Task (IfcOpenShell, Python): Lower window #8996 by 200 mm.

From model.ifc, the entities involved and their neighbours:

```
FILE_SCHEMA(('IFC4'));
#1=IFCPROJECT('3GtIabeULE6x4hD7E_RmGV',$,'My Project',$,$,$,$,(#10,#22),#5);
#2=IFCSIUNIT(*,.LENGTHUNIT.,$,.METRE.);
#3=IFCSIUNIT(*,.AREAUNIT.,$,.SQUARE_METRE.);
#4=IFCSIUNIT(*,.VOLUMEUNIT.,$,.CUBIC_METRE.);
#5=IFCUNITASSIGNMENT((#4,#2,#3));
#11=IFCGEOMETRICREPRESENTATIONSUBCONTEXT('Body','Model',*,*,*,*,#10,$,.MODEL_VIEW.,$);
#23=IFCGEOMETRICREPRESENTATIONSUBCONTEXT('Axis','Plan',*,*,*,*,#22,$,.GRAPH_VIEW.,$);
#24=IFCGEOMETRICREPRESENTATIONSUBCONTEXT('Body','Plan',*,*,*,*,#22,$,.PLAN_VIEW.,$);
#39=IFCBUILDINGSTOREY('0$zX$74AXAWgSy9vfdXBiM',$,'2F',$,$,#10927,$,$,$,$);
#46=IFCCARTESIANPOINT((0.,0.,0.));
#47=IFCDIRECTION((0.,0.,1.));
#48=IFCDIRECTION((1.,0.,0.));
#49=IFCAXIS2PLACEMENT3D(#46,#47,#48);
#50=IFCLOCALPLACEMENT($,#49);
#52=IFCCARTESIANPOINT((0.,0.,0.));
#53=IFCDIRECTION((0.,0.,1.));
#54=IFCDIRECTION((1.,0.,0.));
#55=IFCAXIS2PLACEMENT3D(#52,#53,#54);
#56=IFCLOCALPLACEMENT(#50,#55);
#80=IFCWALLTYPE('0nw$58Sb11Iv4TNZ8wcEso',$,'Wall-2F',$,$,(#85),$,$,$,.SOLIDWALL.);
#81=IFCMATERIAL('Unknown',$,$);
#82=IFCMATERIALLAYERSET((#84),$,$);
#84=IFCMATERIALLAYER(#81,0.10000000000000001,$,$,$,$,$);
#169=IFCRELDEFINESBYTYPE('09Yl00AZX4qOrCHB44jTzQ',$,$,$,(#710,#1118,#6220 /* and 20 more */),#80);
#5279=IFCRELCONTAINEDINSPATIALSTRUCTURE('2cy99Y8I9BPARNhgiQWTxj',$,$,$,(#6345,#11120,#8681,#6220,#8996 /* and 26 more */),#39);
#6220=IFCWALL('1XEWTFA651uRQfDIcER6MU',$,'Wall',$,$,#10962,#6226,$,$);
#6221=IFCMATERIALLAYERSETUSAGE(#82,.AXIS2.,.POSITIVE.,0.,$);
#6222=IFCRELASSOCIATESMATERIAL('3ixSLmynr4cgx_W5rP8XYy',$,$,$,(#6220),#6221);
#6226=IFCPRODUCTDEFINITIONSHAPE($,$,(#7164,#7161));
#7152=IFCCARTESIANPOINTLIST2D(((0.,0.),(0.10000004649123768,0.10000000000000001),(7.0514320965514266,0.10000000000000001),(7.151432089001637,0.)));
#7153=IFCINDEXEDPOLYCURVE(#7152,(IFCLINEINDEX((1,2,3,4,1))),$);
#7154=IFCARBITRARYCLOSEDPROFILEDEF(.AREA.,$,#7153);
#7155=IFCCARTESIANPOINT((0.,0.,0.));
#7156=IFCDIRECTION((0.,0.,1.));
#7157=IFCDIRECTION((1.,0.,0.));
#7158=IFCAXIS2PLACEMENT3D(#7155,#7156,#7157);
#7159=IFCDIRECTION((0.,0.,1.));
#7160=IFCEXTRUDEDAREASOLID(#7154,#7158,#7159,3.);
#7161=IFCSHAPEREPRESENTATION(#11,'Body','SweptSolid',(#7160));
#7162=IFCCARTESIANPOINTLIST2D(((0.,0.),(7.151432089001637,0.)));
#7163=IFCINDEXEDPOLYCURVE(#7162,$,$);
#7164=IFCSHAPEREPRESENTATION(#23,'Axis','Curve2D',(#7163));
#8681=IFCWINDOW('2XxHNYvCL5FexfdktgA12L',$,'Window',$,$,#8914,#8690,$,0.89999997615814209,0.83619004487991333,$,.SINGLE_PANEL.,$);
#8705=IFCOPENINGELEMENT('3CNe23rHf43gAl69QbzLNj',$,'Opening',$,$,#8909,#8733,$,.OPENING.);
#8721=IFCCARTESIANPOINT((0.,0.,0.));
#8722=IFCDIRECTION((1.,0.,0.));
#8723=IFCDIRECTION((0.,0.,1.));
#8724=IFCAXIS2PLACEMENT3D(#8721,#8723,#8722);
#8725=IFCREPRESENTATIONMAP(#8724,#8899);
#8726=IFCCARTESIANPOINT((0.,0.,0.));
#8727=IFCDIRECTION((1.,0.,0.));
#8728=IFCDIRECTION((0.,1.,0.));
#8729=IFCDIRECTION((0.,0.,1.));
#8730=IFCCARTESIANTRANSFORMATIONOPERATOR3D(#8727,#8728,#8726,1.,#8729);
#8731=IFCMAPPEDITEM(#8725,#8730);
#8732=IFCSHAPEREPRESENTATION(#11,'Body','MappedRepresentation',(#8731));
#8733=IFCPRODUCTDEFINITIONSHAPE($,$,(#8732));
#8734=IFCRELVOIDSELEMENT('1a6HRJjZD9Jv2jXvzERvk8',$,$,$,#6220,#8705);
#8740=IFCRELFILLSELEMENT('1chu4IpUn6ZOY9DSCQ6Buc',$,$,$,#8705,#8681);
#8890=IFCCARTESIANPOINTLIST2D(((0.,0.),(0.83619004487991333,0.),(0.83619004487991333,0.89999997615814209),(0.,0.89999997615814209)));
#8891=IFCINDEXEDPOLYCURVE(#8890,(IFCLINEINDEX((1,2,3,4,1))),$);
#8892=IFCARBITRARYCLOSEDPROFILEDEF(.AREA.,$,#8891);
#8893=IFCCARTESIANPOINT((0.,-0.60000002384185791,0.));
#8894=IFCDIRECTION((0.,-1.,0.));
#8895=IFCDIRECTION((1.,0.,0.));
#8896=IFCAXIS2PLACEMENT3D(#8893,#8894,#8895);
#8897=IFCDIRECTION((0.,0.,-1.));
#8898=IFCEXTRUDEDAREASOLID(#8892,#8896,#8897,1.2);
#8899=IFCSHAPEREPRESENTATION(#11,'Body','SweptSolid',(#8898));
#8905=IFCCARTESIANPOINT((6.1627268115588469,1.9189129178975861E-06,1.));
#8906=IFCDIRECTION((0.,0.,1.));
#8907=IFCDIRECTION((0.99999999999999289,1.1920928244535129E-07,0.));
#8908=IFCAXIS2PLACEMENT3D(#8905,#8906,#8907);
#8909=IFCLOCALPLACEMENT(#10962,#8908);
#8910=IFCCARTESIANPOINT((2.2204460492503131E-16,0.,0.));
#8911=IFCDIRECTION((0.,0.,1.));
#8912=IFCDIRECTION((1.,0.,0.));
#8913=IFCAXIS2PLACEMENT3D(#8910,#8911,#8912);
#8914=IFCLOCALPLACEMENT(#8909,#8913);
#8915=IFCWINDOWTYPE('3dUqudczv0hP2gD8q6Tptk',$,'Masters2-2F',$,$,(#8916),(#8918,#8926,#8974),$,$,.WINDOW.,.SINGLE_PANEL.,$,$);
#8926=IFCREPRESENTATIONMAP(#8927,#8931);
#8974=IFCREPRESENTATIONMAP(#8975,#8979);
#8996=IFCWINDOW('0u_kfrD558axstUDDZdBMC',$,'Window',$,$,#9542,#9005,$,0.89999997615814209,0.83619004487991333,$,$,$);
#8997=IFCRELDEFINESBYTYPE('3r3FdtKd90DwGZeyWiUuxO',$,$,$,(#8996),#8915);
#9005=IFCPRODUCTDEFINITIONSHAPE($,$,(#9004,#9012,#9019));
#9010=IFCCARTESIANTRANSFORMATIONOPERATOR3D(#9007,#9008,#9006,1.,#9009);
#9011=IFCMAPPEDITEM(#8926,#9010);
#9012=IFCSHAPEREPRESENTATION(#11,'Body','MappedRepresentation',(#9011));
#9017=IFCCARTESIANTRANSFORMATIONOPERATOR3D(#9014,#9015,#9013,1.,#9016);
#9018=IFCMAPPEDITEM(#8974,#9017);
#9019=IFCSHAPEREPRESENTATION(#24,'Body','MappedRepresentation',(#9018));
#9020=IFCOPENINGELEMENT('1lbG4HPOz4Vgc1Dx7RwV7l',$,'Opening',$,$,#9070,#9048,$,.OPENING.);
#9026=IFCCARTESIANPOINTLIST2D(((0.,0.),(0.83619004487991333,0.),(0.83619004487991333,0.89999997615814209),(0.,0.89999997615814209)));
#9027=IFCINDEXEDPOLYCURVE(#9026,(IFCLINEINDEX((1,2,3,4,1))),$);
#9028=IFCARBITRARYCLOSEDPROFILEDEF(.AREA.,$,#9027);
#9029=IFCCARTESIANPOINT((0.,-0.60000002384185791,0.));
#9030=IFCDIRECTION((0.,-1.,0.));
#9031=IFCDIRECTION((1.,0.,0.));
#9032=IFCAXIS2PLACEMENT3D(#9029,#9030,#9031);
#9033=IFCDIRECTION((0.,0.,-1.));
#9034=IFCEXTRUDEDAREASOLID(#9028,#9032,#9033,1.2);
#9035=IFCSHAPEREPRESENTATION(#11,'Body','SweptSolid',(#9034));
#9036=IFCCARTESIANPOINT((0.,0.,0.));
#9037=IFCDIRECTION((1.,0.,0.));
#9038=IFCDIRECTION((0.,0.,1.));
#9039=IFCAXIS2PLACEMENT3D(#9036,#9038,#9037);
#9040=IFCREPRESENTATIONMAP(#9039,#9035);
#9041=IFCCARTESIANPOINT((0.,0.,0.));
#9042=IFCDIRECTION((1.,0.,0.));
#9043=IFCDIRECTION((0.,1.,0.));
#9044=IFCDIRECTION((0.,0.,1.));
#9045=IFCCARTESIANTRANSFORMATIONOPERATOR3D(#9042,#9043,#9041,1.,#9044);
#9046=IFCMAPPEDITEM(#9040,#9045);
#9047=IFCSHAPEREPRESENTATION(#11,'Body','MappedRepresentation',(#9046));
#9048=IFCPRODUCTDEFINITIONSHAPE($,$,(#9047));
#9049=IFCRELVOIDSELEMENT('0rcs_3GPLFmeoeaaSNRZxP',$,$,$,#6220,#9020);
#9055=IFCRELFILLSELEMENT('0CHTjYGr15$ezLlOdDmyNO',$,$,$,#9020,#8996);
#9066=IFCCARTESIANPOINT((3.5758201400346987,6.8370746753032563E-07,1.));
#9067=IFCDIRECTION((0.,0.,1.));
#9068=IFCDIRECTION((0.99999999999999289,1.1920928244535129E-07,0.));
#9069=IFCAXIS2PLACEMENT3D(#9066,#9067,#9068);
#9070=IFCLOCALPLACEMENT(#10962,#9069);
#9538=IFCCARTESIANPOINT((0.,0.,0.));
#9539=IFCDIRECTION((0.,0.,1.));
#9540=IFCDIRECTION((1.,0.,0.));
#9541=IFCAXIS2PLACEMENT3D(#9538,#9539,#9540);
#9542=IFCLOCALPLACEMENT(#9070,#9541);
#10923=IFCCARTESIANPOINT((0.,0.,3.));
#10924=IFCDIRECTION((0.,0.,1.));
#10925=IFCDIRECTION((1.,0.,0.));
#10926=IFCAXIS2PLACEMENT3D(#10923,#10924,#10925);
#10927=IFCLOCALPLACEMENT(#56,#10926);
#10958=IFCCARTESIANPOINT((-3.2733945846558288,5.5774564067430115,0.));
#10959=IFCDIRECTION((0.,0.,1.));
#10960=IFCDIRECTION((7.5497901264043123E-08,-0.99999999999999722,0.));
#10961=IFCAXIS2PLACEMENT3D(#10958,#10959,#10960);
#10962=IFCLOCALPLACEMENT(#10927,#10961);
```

```python
import numpy as np
import ifcopenshell
import ifcopenshell.api.geometry
import ifcopenshell.util.placement
import ifcopenshell.util.unit

model = ifcopenshell.open("model.ifc")
unit_scale = ifcopenshell.util.unit.calculate_unit_scale(model)

window = model.by_id(8996)
opening = window.FillsVoids[0].RelatingOpeningElement
dz = -0.2 / unit_scale

shift = np.array([0.0, 0.0, dz])
# The window is placed relative to its opening, so it follows when the opening moves.
matrix = ifcopenshell.util.placement.get_local_placement(opening.ObjectPlacement)
matrix[:3, 3] += shift
ifcopenshell.api.geometry.edit_object_placement(
    model, product=opening, matrix=matrix, is_si=False, should_transform_children=True
)

print(f"moved by {dz * unit_scale:+.3f} m")

model.write("model_v2.ifc")
```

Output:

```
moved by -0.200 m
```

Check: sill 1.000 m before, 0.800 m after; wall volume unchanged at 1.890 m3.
